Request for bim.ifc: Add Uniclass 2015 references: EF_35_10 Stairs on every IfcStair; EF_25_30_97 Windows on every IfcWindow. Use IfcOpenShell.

First a look at what the model holds.

```python
import ifcopenshell

model = ifcopenshell.open("bim.ifc")
print(model.schema)
print("classifications:", [c.Name for c in model.by_type("IfcClassification")])
for ifc_class in ("IfcDoor", "IfcRoof", "IfcStair", "IfcWall", "IfcWindow"):
    print(ifc_class, len(model.by_type(ifc_class)))
```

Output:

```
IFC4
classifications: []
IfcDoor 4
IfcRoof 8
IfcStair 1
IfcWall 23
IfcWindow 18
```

```python
import ifcopenshell
import ifcopenshell.api.classification

model = ifcopenshell.open("bim.ifc")

system = ifcopenshell.api.classification.add_classification(model, classification="Uniclass 2015")

codes = {
    "IfcStair": ("EF_35_10", "Stairs"),
    "IfcWindow": ("EF_25_30_97", "Windows"),
}
for ifc_class, (code, name) in codes.items():
    products = model.by_type(ifc_class)
    ifcopenshell.api.classification.add_reference(
        model, products=products, classification=system, identification=code, name=name
    )
    print(code, len(products))

model.write("bim-out.ifc")
```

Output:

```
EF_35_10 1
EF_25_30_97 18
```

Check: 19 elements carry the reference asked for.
